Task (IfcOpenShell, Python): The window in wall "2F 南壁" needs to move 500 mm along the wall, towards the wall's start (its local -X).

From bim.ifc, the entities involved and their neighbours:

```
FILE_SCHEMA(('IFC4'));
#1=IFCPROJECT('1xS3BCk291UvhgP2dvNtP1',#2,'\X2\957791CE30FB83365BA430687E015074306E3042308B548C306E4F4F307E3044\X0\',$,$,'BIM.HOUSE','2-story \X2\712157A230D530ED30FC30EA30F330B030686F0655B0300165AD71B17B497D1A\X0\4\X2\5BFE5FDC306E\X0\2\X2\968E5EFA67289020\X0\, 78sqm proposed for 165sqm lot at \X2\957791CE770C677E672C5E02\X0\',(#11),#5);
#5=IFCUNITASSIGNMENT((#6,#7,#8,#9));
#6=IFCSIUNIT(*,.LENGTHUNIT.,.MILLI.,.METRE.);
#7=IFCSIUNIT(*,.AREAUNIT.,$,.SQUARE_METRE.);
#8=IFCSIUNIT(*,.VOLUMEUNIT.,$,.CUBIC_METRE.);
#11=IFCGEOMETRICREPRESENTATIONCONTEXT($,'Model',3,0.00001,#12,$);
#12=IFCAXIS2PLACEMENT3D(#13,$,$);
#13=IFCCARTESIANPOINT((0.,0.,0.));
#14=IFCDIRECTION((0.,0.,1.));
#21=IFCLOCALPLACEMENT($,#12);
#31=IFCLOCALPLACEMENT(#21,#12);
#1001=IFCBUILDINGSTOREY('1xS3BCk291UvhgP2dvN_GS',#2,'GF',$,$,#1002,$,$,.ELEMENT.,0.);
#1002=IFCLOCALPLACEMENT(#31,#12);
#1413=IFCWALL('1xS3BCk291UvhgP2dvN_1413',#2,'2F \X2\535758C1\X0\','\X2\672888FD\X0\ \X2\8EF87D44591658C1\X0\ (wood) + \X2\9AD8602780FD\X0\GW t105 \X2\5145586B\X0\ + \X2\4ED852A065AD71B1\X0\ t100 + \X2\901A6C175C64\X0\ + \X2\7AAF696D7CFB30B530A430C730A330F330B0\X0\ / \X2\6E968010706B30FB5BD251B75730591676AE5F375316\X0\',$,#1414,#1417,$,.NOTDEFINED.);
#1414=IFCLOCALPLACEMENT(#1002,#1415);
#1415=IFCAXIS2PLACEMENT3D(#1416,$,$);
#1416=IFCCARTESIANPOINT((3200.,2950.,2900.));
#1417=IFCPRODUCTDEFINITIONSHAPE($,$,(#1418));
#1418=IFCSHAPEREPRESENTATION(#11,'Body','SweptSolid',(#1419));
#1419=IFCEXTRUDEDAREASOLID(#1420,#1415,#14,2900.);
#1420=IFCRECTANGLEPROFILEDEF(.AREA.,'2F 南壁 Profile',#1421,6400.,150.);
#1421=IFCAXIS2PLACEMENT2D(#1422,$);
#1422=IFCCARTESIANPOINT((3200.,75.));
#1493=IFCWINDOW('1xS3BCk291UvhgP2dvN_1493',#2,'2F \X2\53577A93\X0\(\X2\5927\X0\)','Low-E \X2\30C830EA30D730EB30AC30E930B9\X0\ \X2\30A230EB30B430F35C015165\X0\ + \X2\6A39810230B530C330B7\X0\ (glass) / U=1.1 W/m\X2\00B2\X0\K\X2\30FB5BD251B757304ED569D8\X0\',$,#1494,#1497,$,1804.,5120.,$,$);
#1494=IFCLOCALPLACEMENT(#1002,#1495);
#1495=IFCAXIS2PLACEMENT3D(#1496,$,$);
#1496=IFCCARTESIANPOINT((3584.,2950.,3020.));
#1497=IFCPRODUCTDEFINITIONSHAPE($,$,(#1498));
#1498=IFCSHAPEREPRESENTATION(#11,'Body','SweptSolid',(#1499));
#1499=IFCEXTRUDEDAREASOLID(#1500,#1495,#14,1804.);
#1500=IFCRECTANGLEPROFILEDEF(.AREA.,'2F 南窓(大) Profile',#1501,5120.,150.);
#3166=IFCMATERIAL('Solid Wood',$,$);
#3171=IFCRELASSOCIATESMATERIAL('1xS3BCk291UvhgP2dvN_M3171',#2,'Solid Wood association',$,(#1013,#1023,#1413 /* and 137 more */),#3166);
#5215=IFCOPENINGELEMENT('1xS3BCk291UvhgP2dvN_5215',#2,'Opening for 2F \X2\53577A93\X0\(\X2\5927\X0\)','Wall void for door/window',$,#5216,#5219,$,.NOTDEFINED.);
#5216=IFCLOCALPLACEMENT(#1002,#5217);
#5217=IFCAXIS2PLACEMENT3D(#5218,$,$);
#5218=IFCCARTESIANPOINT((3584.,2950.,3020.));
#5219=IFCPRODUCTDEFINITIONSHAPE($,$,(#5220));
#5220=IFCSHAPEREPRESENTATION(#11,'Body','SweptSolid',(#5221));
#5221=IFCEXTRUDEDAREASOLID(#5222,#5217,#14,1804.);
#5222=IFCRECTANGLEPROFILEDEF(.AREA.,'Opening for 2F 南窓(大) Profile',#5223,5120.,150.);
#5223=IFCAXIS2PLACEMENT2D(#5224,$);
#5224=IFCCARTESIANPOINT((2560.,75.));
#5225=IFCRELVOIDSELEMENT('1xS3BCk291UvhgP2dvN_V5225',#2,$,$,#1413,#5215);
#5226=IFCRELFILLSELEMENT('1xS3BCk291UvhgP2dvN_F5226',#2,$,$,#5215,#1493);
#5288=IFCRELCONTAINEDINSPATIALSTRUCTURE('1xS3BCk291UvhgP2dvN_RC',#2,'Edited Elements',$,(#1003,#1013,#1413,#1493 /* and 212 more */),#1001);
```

```python
import ifcopenshell
import ifcopenshell.api.geometry
import ifcopenshell.util.placement
import ifcopenshell.util.unit

model = ifcopenshell.open("bim.ifc")
unit_scale = ifcopenshell.util.unit.calculate_unit_scale(model)

window = model.by_guid("1xS3BCk291UvhgP2dvN_1493")
opening = window.FillsVoids[0].RelatingOpeningElement
wall = opening.VoidsElements[0].RelatingBuildingElement

wall_matrix = ifcopenshell.util.placement.get_local_placement(wall.ObjectPlacement)
shift = wall_matrix[:3, 0] * -0.5 / unit_scale
before = ifcopenshell.util.placement.get_local_placement(window.ObjectPlacement)[:3, 3].copy()

# The window is not placed relative to its opening, so move both.
for product in (opening, window):
    matrix = ifcopenshell.util.placement.get_local_placement(product.ObjectPlacement)
    matrix[:3, 3] += shift
    ifcopenshell.api.geometry.edit_object_placement(model, product=product, matrix=matrix, is_si=False)

after = ifcopenshell.util.placement.get_local_placement(window.ObjectPlacement)[:3, 3]
print("window moved by", (after - before).round(3) + 0.0)

model.write("bim_rev.ifc")
```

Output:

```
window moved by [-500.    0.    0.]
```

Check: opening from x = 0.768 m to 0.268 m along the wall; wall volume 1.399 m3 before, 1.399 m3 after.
